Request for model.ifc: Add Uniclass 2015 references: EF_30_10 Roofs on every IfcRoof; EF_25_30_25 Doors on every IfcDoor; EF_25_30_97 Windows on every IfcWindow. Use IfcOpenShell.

First a look at what the model holds.

```python
import ifcopenshell

model = ifcopenshell.open("model.ifc")
print(model.schema)
print("classifications:", [c.Name for c in model.by_type("IfcClassification")])
for ifc_class in ("IfcDoor", "IfcRoof", "IfcStair", "IfcWall", "IfcWindow"):
    print(ifc_class, len(model.by_type(ifc_class)))
```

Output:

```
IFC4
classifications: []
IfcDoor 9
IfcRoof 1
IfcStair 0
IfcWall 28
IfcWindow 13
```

```python
import ifcopenshell
import ifcopenshell.api.classification

model = ifcopenshell.open("model.ifc")

system = ifcopenshell.api.classification.add_classification(model, classification="Uniclass 2015")

codes = {
    "IfcRoof": ("EF_30_10", "Roofs"),
    "IfcDoor": ("EF_25_30_25", "Doors"),
    "IfcWindow": ("EF_25_30_97", "Windows"),
}
for ifc_class, (code, name) in codes.items():
    products = model.by_type(ifc_class)
    ifcopenshell.api.classification.add_reference(
        model, products=products, classification=system, identification=code, name=name
    )
    print(code, len(products))

model.write("model_updated.ifc")
```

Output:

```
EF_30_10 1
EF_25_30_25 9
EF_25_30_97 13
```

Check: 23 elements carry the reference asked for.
